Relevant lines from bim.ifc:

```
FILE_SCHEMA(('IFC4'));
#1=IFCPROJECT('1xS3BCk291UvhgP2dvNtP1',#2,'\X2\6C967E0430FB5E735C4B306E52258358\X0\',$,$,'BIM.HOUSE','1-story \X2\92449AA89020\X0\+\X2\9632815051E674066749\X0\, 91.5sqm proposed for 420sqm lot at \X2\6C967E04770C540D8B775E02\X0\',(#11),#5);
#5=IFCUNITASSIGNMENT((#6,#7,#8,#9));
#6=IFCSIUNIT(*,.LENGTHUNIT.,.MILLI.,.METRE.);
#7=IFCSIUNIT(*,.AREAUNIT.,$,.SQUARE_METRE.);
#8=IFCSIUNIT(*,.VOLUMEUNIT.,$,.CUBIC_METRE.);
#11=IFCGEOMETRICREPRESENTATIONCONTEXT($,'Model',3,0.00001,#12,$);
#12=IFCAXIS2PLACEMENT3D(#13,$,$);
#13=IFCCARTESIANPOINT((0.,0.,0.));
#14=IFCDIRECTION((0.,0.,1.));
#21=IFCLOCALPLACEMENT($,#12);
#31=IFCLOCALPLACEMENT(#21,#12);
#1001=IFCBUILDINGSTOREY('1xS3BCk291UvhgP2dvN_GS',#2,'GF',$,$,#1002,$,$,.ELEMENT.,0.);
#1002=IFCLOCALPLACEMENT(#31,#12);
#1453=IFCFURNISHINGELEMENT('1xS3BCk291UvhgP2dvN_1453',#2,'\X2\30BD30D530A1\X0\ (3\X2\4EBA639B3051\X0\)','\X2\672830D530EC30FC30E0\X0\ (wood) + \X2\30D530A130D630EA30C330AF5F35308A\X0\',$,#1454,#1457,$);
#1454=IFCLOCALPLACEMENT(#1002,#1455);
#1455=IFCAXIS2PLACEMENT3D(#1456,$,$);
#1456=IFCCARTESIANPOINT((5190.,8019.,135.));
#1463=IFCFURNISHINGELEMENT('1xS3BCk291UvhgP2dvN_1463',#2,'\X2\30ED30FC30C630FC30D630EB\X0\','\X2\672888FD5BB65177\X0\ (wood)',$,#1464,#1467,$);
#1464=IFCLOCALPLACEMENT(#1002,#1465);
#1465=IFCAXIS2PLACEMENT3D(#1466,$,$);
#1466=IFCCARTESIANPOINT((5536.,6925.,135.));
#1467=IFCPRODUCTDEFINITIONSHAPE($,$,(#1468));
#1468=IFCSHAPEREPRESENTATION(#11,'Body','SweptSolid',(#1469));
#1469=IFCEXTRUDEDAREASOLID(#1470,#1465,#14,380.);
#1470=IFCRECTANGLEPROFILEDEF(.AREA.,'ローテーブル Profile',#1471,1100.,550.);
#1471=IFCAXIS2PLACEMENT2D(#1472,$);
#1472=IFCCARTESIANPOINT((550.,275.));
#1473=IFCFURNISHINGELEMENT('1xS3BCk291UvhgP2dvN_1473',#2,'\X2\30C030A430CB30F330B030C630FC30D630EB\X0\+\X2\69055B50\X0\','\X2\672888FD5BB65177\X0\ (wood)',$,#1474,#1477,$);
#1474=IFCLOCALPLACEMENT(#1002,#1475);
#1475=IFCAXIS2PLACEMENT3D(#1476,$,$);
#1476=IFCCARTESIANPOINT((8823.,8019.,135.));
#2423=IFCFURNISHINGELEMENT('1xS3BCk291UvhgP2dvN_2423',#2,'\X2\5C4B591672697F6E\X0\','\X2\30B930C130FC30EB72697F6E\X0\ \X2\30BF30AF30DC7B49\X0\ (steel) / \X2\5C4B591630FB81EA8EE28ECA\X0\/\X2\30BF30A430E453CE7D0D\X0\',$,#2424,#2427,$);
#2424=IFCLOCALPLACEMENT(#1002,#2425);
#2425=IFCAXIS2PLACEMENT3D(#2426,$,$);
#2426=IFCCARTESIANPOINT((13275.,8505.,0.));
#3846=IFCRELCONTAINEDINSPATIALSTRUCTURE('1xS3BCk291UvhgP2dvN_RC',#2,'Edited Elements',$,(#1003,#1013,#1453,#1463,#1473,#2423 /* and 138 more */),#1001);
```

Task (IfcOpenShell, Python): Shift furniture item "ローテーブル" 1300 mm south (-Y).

```python
import ifcopenshell
import ifcopenshell.api.geometry
import ifcopenshell.util.placement

model = ifcopenshell.open("bim.ifc")

item = model.by_guid("1xS3BCk291UvhgP2dvN_1463")
matrix = ifcopenshell.util.placement.get_local_placement(item.ObjectPlacement)
matrix[1, 3] -= 1300.0
ifcopenshell.api.geometry.edit_object_placement(model, product=item, matrix=matrix, is_si=False)

print(ifcopenshell.util.placement.get_local_placement(item.ObjectPlacement).round(3) + 0.0)

model.write("bim_edited.ifc")
```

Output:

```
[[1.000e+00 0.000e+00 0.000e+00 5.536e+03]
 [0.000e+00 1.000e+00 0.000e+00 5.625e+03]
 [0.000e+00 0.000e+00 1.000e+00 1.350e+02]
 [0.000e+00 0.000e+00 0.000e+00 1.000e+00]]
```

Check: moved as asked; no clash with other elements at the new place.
